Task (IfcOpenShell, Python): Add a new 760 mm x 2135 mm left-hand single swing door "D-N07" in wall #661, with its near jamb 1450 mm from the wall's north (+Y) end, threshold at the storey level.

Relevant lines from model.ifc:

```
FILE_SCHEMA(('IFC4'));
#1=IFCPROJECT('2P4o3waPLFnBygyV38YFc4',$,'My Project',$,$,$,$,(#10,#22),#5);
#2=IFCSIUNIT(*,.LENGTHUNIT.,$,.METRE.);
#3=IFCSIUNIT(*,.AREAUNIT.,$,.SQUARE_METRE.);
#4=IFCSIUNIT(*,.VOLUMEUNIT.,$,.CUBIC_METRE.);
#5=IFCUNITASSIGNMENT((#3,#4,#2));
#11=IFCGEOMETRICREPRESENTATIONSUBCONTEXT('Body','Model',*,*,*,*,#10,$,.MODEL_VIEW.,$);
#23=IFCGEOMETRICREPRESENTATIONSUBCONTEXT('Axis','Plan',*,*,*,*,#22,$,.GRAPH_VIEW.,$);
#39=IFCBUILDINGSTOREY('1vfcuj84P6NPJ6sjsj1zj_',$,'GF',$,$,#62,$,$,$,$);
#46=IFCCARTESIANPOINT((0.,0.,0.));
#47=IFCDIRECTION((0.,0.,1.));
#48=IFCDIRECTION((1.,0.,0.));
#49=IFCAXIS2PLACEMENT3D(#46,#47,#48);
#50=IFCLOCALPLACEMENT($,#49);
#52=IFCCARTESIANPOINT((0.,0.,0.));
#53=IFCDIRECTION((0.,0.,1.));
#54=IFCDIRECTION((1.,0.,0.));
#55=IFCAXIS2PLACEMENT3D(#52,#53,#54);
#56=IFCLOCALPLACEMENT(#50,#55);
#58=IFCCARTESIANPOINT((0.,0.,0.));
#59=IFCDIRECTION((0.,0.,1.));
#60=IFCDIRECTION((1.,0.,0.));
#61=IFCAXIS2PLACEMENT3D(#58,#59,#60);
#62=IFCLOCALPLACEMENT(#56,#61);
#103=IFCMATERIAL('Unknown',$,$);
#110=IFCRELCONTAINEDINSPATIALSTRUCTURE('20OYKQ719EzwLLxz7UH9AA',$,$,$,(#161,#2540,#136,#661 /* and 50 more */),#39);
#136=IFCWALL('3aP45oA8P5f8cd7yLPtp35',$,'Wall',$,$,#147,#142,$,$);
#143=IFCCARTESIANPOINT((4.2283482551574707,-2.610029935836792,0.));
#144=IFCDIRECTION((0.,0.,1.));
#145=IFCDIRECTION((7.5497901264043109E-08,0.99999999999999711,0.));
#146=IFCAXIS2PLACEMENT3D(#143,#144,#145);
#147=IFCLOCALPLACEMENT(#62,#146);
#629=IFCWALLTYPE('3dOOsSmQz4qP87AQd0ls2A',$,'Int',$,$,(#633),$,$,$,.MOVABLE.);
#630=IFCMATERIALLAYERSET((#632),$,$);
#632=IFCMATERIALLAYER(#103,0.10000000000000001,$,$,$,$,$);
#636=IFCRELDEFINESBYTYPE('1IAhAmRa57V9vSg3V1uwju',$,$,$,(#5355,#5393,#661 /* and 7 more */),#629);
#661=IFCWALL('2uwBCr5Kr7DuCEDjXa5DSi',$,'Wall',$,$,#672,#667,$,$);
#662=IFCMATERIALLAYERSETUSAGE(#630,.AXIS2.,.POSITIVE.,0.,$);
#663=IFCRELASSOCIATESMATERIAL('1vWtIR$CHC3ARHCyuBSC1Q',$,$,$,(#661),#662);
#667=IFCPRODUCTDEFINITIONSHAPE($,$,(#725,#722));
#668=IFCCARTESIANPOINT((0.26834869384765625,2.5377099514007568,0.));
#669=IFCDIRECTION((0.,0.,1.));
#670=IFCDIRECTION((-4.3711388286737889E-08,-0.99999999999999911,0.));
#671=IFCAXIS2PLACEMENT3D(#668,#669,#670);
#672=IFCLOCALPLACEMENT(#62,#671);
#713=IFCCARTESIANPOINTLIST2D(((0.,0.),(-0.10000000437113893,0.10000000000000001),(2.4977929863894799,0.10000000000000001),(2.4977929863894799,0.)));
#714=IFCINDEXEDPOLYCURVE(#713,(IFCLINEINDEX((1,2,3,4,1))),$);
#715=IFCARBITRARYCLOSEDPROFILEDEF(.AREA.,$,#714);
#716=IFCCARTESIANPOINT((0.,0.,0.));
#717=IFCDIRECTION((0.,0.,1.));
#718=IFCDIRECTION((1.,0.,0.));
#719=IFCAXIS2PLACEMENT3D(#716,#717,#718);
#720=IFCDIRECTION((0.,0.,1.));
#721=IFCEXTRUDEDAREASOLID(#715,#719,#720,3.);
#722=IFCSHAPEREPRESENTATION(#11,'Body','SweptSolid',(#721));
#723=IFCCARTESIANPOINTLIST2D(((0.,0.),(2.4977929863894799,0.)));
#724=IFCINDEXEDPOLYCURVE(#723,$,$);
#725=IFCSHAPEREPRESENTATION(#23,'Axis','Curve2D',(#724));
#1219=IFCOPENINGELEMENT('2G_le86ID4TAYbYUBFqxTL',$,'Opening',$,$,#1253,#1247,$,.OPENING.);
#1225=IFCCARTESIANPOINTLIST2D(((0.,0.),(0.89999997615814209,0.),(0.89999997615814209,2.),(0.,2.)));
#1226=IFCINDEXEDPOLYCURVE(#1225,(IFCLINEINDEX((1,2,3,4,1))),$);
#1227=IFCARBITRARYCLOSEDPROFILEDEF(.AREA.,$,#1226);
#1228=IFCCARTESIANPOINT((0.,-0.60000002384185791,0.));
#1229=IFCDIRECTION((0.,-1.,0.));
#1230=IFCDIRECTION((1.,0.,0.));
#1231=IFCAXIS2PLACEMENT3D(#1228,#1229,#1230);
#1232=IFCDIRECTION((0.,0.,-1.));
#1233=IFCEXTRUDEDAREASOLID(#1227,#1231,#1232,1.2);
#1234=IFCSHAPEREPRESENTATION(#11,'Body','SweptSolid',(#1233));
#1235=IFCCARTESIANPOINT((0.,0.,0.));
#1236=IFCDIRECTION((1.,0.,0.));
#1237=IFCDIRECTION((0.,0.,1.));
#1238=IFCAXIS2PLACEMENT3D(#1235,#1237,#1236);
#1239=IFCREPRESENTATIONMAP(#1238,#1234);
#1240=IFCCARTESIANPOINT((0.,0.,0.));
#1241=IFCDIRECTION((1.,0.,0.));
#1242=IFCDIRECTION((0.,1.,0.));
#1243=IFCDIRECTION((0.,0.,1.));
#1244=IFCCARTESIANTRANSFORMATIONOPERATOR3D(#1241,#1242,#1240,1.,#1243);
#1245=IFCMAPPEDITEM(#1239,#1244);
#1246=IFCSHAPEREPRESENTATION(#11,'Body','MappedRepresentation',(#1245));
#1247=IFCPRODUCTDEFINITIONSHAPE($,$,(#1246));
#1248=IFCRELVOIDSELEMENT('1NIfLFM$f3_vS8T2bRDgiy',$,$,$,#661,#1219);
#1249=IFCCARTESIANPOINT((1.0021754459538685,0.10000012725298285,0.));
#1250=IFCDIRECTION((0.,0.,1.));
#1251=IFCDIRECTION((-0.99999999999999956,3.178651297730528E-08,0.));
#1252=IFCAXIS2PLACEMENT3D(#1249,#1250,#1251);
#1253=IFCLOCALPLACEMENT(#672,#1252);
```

```python
import numpy as np
import ifcopenshell
import ifcopenshell.api.feature
import ifcopenshell.api.geometry
import ifcopenshell.api.root
import ifcopenshell.api.spatial
import ifcopenshell.geom
import ifcopenshell.util.element
import ifcopenshell.util.placement
import ifcopenshell.util.representation
import ifcopenshell.util.shape
import ifcopenshell.util.unit

model = ifcopenshell.open("model.ifc")
unit_scale = ifcopenshell.util.unit.calculate_unit_scale(model)
settings = ifcopenshell.geom.settings()


def volume(element):
    """Net volume in cubic metres, openings subtracted."""
    shape = ifcopenshell.geom.create_shape(settings, element)
    return ifcopenshell.util.shape.get_volume(shape.geometry)


wall = model.by_guid("2uwBCr5Kr7DuCEDjXa5DSi")
storey = ifcopenshell.util.element.get_container(wall, ifc_class="IfcBuildingStorey")
context = ifcopenshell.util.representation.get_context(model, "Model", "Body", "MODEL_VIEW")
before = volume(wall)

width, height, from_end, sill = 0.76, 2.135, 1.45, 0.0  # metres

# The wall runs along its own X axis, and the end named is its -X end.
wall_shape = ifcopenshell.geom.create_shape(settings, wall)
x, y, z = ifcopenshell.util.shape.get_vertices(wall_shape.geometry).T
start = x.min() + from_end
face, thickness = float(y.min()), float(y.max() - y.min())
wall_matrix = ifcopenshell.util.placement.get_local_placement(wall.ObjectPlacement)
level = ifcopenshell.util.placement.get_local_placement(storey.ObjectPlacement)[2, 3]


def in_wall(x, y):
    """Placement at x, y metres in the wall's axes, at sill height."""
    matrix = wall_matrix.copy()
    matrix[:, 3] = wall_matrix @ np.array([x / unit_scale, y / unit_scale, 0.0, 1.0])
    matrix[2, 3] = level + sill / unit_scale
    return matrix


# Opening: a box that overshoots both wall faces by 50 mm.
opening = ifcopenshell.api.root.create_entity(model, ifc_class="IfcOpeningElement", predefined_type="OPENING")
box = ifcopenshell.api.geometry.add_wall_representation(
    model, context=context, length=width, height=height, thickness=thickness + 0.1
)
ifcopenshell.api.geometry.assign_representation(model, product=opening, representation=box)
ifcopenshell.api.geometry.edit_object_placement(model, product=opening, matrix=in_wall(start, face - 0.05), is_si=False)
ifcopenshell.api.feature.add_feature(model, feature=opening, element=wall)

door = ifcopenshell.api.root.create_entity(model, ifc_class="IfcDoor", name="D-N07", predefined_type="DOOR")
door.OverallWidth, door.OverallHeight = width / unit_scale, height / unit_scale
door.OperationType = "SINGLE_SWING_LEFT"
body = ifcopenshell.api.geometry.add_door_representation(
    model,
    context=context,
    overall_width=door.OverallWidth,
    overall_height=door.OverallHeight,
    operation_type="SINGLE_SWING_LEFT",
    lining_properties={"LiningDepth": thickness / unit_scale, "ThresholdDepth": thickness / unit_scale},
)
ifcopenshell.api.geometry.assign_representation(model, product=door, representation=body)
ifcopenshell.api.spatial.assign_container(model, products=[door], relating_structure=storey)
ifcopenshell.api.feature.add_filling(model, opening=opening, element=door)

# The lining spans the wall, so the door starts at the wall face.
ifcopenshell.api.geometry.edit_object_placement(model, product=door, matrix=in_wall(start, face), is_si=False)

after = volume(wall)

print(f"wall volume {before:.3f} -> {after:.3f} m3")

model.write("model-out.ifc")
```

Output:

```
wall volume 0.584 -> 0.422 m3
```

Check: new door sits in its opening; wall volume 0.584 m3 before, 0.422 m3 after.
